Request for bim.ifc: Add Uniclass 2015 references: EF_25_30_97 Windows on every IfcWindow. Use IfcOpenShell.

First a look at what the model holds.

```python
import ifcopenshell

model = ifcopenshell.open("bim.ifc")
print(model.schema)
print("classifications:", [c.Name for c in model.by_type("IfcClassification")])
for ifc_class in ("IfcDoor", "IfcRoof", "IfcStair", "IfcWall", "IfcWindow"):
    print(ifc_class, len(model.by_type(ifc_class)))
```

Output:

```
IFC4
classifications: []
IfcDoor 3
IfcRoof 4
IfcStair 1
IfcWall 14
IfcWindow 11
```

```python
import ifcopenshell
import ifcopenshell.api.classification

model = ifcopenshell.open("bim.ifc")

system = ifcopenshell.api.classification.add_classification(model, classification="Uniclass 2015")

codes = {
    "IfcWindow": ("EF_25_30_97", "Windows"),
}
for ifc_class, (code, name) in codes.items():
    products = model.by_type(ifc_class)
    ifcopenshell.api.classification.add_reference(
        model, products=products, classification=system, identification=code, name=name
    )
    print(code, len(products))

model.write("bim_edited.ifc")
```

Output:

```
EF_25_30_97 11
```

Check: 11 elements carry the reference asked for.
